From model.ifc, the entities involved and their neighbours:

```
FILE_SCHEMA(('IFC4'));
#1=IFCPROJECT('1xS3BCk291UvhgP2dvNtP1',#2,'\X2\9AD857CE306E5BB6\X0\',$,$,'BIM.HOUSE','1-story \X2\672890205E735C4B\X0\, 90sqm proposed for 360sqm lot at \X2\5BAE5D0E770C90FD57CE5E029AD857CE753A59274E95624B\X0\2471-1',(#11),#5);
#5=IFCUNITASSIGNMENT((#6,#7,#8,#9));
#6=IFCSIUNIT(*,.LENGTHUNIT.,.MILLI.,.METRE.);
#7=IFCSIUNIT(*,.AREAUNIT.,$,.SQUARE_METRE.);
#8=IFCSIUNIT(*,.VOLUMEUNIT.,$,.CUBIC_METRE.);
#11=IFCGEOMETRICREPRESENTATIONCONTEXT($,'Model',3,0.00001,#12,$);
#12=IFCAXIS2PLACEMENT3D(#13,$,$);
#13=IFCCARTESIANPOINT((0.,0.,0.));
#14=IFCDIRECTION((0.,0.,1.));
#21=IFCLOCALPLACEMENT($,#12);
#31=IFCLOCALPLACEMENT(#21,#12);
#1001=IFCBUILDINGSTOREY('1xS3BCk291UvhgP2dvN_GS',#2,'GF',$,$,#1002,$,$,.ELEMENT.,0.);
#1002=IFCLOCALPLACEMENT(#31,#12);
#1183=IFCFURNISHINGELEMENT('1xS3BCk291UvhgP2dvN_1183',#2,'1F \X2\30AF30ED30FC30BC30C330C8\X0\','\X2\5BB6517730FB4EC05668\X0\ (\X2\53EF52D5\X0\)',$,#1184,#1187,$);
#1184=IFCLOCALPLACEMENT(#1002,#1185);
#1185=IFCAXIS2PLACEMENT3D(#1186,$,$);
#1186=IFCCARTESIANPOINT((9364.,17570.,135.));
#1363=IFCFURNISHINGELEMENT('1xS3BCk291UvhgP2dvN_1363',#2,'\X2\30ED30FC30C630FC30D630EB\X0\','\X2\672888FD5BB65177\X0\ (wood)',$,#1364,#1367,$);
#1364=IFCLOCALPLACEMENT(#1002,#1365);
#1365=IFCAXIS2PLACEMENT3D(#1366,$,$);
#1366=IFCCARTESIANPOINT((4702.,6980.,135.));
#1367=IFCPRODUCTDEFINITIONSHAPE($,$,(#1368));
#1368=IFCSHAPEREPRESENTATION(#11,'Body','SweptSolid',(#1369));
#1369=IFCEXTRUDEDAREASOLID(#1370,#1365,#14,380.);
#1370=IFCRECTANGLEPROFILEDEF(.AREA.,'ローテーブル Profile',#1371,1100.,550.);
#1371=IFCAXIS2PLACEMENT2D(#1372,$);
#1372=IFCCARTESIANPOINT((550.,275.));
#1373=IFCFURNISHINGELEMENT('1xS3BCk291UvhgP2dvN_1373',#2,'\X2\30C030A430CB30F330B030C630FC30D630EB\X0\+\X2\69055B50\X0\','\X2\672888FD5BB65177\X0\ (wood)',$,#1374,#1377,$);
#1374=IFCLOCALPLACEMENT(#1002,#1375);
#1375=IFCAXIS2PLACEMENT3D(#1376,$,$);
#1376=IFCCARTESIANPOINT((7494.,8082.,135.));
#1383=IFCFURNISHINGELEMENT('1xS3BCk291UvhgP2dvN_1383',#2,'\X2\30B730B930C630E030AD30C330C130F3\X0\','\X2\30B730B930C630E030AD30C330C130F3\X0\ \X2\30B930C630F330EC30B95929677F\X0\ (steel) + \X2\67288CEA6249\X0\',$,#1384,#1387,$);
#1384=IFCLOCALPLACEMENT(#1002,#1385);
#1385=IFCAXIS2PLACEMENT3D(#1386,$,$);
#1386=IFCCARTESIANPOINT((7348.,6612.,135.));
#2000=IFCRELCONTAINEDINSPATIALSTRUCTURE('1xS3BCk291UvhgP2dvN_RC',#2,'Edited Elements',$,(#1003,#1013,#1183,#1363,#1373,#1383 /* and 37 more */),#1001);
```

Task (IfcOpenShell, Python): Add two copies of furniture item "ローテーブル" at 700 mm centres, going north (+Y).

```python
import numpy as np
import ifcopenshell
import ifcopenshell.api.geometry
import ifcopenshell.api.root
import ifcopenshell.util.element
import ifcopenshell.util.placement
import ifcopenshell.util.unit

model = ifcopenshell.open("model.ifc")
unit_scale = ifcopenshell.util.unit.calculate_unit_scale(model)


def reuse_history(source, copy):
    """copy_class also copies each property set's owner history, people and application; keep the originals."""
    for rel in copy.IsDefinedBy:
        if rel.is_a("IfcRelDefinesByProperties") and (history := rel.RelatingPropertyDefinition.OwnerHistory):
            rel.RelatingPropertyDefinition.OwnerHistory = source.OwnerHistory
            ifcopenshell.util.element.remove_deep2(model, history)


source = model.by_guid("1xS3BCk291UvhgP2dvN_1363")
base = ifcopenshell.util.placement.get_local_placement(source.ObjectPlacement)
step = np.array([0.0, 1.0, 0.0]) * 0.7 / unit_scale

for i in range(1, 3):
    copy = ifcopenshell.api.root.copy_class(model, product=source)
    copy.Representation = ifcopenshell.util.element.copy_deep(
        model, source.Representation, exclude=["IfcGeometricRepresentationContext", "IfcRepresentationMap"]
    )
    reuse_history(source, copy)
    matrix = base.copy()
    matrix[:3, 3] += i * step
    print("added at", matrix[:3, 3].round(3) + 0.0)
    ifcopenshell.api.geometry.edit_object_placement(model, product=copy, matrix=matrix, is_si=False)

model.write("model_rev.ifc")
```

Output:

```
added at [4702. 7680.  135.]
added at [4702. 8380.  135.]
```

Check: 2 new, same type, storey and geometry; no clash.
